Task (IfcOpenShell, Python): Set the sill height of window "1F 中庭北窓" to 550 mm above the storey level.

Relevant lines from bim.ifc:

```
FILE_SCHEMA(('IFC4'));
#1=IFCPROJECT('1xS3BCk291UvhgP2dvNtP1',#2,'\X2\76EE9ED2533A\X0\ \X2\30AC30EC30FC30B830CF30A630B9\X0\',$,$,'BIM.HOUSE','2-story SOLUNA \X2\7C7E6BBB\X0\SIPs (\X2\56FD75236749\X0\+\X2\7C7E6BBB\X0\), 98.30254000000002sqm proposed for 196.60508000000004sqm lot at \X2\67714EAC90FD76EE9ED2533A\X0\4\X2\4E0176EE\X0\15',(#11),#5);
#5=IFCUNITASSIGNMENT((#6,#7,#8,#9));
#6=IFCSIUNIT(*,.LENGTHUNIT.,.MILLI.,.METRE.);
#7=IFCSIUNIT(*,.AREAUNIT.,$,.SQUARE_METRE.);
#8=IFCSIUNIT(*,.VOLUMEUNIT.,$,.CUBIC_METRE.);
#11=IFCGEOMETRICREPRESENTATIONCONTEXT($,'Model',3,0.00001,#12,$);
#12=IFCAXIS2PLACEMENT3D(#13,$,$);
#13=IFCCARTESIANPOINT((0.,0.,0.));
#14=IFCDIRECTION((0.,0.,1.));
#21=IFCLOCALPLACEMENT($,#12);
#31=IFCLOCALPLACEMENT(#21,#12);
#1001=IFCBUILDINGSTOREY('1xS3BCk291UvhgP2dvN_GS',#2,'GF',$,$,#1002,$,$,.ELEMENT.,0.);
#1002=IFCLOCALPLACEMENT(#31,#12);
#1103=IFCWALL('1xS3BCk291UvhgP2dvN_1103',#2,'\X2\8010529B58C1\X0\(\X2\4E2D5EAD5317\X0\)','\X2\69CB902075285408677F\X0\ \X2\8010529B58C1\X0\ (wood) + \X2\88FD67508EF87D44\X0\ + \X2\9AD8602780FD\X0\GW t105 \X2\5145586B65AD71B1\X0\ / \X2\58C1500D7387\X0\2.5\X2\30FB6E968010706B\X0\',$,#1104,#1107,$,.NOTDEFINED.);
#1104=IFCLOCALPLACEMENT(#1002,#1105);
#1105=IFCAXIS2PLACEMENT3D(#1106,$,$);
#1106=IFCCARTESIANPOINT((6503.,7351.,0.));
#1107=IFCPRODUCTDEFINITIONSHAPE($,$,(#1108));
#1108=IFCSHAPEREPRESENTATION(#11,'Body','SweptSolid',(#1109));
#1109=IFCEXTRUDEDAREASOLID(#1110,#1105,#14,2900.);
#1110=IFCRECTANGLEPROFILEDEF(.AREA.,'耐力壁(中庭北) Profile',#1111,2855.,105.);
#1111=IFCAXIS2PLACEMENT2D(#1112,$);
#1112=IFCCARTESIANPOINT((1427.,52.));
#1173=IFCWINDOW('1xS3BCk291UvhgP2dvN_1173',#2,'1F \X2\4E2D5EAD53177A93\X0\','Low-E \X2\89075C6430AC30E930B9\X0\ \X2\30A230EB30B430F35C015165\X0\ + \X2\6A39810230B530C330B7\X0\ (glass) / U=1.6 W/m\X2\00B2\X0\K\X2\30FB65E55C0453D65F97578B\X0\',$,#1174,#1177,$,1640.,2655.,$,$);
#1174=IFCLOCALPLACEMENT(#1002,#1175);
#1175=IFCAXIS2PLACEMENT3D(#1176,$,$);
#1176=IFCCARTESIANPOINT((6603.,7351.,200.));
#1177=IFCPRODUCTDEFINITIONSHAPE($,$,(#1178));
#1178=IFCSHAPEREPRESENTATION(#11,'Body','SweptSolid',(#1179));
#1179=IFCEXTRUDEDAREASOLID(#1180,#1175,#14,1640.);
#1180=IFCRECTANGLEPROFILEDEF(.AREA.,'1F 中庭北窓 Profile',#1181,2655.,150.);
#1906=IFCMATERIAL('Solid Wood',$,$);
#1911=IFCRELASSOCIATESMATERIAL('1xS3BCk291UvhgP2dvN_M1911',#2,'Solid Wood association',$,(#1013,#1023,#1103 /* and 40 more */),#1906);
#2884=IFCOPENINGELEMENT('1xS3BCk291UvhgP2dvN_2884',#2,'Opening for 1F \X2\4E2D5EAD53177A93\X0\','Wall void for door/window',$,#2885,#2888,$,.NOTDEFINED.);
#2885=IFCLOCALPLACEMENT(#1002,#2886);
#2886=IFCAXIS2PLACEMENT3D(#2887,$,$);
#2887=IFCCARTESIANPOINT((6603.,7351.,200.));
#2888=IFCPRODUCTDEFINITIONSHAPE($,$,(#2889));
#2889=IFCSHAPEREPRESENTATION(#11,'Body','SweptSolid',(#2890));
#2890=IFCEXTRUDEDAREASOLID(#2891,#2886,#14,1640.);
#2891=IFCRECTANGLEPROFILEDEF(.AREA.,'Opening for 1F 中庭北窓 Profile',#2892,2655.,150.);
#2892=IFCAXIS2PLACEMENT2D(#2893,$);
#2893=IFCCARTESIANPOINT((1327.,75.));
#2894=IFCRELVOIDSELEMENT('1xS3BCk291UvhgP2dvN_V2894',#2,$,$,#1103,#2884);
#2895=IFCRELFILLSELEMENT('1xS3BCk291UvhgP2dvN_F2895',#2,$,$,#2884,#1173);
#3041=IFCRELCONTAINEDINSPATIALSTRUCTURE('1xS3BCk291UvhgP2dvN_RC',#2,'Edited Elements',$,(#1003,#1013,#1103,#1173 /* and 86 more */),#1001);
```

```python
import numpy as np
import ifcopenshell
import ifcopenshell.api.geometry
import ifcopenshell.geom
import ifcopenshell.util.element
import ifcopenshell.util.placement
import ifcopenshell.util.shape
import ifcopenshell.util.unit

model = ifcopenshell.open("bim.ifc")
unit_scale = ifcopenshell.util.unit.calculate_unit_scale(model)

window = model.by_guid("1xS3BCk291UvhgP2dvN_1173")
opening = window.FillsVoids[0].RelatingOpeningElement
storey = ifcopenshell.util.element.get_container(window, ifc_class="IfcBuildingStorey")
level = ifcopenshell.util.placement.get_local_placement(storey.ObjectPlacement)[2, 3]

# The opening's origin need not be at the sill, so measure its lowest point.
shape = ifcopenshell.geom.create_shape(ifcopenshell.geom.settings(), opening)
bottom = ifcopenshell.util.shape.get_shape_bottom_elevation(shape, shape.geometry) / unit_scale
dz = level + 0.55 / unit_scale - bottom

shift = np.array([0.0, 0.0, dz])
# The window is not placed relative to its opening, so move both.
for product in (opening, window):
    matrix = ifcopenshell.util.placement.get_local_placement(product.ObjectPlacement)
    matrix[:3, 3] += shift
    ifcopenshell.api.geometry.edit_object_placement(model, product=product, matrix=matrix, is_si=False)

print(f"moved by {dz * unit_scale:+.3f} m")

model.write("bim_v2.ifc")
```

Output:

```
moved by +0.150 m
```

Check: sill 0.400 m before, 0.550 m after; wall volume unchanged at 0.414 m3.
